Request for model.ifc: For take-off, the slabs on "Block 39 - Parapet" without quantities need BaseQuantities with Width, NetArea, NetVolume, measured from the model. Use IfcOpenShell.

First a look at what the model holds.

```python
import ifcopenshell
import ifcopenshell.util.element
import ifcopenshell.util.unit

model = ifcopenshell.open("model.ifc")
print(model.schema)
for unit_type in ("LENGTHUNIT", "AREAUNIT", "VOLUMEUNIT"):
    print(unit_type, ifcopenshell.util.unit.calculate_unit_scale(model, unit_type))
storey = next(s for s in model.by_type("IfcBuildingStorey") if s.Name == "Block 39 - Parapet")
slabs = [e for e in ifcopenshell.util.element.get_decomposition(storey) if e.is_a("IfcSlab")]
for e in sorted(slabs, key=lambda e: e.id()):
    print(e.id(), e.is_a(), e.Name, list(ifcopenshell.util.element.get_psets(e, qtos_only=True)), sep=" | ")
```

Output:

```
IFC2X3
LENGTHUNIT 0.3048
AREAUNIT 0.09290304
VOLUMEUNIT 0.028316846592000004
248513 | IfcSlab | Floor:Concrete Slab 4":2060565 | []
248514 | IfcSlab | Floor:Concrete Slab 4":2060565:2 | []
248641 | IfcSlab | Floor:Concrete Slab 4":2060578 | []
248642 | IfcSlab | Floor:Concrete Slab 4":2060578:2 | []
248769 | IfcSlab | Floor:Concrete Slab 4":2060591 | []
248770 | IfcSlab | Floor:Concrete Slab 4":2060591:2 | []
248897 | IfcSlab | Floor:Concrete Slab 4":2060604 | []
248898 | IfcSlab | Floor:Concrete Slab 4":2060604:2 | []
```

```python
import ifcopenshell
import ifcopenshell.api.pset
import ifcopenshell.geom
import ifcopenshell.util.element
import ifcopenshell.util.shape
import ifcopenshell.util.unit

model = ifcopenshell.open("model.ifc")
unit_scale = ifcopenshell.util.unit.calculate_unit_scale(model)
area_scale = ifcopenshell.util.unit.calculate_unit_scale(model, "AREAUNIT")
volume_scale = ifcopenshell.util.unit.calculate_unit_scale(model, "VOLUMEUNIT")
settings = ifcopenshell.geom.settings()

storey = next(s for s in model.by_type("IfcBuildingStorey") if s.Name == "Block 39 - Parapet")
slabs = [e for e in ifcopenshell.util.element.get_decomposition(storey) if e.is_a("IfcSlab")]

for e in sorted(slabs, key=lambda e: e.id()):
    if ifcopenshell.util.element.get_psets(e, qtos_only=True, should_inherit=False):
        continue
    # Geometry comes back in metres, in the element's own axes.
    shape = ifcopenshell.geom.create_shape(settings, e)
    values = {
        "Width": ifcopenshell.util.shape.get_z(shape.geometry) / unit_scale,
        "NetArea": ifcopenshell.util.shape.get_footprint_area(shape.geometry) / area_scale,
        "NetVolume": ifcopenshell.util.shape.get_volume(shape.geometry) / volume_scale,
    }
    qto = ifcopenshell.api.pset.add_qto(model, product=e, name="BaseQuantities")
    ifcopenshell.api.pset.edit_qto(model, qto=qto, properties=values)
    print(e.id(), {k: round(v, 3) for k, v in values.items()})

model.write("model_edited.ifc")
```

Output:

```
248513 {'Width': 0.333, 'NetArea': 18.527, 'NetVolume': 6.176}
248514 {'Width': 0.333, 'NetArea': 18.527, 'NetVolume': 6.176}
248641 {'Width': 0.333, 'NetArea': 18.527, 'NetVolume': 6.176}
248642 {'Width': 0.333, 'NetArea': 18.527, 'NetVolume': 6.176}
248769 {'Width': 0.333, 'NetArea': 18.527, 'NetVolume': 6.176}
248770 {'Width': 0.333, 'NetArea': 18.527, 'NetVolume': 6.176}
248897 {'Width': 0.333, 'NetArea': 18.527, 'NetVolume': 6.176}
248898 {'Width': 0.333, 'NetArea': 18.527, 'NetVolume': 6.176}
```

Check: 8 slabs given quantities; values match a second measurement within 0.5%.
